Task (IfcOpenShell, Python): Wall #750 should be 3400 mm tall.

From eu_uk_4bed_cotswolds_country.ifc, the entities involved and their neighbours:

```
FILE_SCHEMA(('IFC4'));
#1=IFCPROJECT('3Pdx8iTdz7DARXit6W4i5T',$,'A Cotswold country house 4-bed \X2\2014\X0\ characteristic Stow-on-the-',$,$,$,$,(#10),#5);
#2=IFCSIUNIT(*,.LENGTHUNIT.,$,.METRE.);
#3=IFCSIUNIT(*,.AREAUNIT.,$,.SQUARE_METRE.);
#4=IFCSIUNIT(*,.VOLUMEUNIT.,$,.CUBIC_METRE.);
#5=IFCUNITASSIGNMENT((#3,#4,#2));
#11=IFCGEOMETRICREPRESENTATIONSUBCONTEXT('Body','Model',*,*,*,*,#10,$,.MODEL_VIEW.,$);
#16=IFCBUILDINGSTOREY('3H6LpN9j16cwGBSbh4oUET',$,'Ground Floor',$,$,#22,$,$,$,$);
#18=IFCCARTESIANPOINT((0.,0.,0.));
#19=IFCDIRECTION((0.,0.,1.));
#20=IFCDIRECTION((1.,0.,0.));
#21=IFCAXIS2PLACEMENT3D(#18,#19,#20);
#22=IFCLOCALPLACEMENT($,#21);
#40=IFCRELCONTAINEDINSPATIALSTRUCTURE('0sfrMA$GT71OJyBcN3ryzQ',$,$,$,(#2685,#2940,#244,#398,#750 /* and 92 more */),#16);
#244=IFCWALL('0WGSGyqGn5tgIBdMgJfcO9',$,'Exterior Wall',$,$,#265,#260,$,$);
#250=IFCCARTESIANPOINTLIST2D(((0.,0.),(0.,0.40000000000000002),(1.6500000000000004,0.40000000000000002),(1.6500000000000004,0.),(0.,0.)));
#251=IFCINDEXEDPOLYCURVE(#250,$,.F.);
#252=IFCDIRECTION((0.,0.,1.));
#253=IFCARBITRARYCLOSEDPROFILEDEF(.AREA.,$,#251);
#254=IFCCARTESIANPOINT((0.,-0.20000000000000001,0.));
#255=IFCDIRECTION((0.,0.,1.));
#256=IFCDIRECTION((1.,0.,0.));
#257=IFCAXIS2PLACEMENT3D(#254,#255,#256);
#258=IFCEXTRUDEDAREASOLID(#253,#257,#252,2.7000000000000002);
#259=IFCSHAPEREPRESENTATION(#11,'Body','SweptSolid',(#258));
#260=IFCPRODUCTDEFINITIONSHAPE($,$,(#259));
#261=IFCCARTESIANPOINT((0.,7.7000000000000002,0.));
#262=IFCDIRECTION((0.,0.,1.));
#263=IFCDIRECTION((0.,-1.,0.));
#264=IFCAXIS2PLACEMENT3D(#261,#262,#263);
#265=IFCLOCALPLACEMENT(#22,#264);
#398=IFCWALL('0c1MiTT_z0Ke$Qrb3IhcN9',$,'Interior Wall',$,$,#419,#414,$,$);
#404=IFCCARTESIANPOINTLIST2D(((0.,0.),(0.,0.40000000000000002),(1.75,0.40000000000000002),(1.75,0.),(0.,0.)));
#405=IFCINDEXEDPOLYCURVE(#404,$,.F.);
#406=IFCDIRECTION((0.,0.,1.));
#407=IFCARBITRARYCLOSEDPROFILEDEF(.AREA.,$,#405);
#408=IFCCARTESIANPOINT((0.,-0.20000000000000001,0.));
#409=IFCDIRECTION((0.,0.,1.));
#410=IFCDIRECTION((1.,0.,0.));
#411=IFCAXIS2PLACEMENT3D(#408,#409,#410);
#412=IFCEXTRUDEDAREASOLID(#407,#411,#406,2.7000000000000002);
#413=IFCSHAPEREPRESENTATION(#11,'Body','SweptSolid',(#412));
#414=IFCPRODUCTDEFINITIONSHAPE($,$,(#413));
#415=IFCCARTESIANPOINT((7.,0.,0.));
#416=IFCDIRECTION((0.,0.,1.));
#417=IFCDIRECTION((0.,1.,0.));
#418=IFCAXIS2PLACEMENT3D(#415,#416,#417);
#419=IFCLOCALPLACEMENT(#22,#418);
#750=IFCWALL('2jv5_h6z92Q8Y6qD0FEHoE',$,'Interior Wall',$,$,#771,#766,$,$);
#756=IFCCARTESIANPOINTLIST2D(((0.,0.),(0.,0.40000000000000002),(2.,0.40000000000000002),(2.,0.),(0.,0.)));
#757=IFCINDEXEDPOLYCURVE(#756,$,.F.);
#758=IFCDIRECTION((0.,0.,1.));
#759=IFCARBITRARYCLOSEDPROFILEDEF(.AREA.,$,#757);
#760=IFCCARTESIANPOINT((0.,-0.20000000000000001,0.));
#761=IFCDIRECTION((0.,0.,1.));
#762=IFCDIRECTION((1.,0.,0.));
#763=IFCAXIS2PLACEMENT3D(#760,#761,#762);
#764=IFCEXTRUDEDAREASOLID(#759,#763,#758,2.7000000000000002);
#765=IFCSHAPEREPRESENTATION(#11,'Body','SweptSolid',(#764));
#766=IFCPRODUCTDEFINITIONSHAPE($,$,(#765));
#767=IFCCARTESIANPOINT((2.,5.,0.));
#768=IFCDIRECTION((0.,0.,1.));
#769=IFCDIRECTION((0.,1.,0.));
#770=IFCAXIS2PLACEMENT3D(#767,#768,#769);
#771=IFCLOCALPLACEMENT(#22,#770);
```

```python
import ifcopenshell
import ifcopenshell.geom
import ifcopenshell.util.representation
import ifcopenshell.util.shape
import ifcopenshell.util.unit

model = ifcopenshell.open("eu_uk_4bed_cotswolds_country.ifc")
unit_scale = ifcopenshell.util.unit.calculate_unit_scale(model)
settings = ifcopenshell.geom.settings()


def volume(element):
    """Net volume in cubic metres, openings subtracted."""
    shape = ifcopenshell.geom.create_shape(settings, element)
    return ifcopenshell.util.shape.get_volume(shape.geometry)


wall = model.by_guid("2jv5_h6z92Q8Y6qD0FEHoE")
before = volume(wall)

body = ifcopenshell.util.representation.get_representation(wall, "Model", "Body")
solid = body.Items[0]
old_height = solid.Depth
solid.Depth = 3.4 / unit_scale
after = volume(wall)

print(f"height {old_height:g} -> {solid.Depth:g}, volume {before:.3f} -> {after:.3f} m3")

model.write("eu_uk_4bed_cotswolds_country_updated.ifc")
```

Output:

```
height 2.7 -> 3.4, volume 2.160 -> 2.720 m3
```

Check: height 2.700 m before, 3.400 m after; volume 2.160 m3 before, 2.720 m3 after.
